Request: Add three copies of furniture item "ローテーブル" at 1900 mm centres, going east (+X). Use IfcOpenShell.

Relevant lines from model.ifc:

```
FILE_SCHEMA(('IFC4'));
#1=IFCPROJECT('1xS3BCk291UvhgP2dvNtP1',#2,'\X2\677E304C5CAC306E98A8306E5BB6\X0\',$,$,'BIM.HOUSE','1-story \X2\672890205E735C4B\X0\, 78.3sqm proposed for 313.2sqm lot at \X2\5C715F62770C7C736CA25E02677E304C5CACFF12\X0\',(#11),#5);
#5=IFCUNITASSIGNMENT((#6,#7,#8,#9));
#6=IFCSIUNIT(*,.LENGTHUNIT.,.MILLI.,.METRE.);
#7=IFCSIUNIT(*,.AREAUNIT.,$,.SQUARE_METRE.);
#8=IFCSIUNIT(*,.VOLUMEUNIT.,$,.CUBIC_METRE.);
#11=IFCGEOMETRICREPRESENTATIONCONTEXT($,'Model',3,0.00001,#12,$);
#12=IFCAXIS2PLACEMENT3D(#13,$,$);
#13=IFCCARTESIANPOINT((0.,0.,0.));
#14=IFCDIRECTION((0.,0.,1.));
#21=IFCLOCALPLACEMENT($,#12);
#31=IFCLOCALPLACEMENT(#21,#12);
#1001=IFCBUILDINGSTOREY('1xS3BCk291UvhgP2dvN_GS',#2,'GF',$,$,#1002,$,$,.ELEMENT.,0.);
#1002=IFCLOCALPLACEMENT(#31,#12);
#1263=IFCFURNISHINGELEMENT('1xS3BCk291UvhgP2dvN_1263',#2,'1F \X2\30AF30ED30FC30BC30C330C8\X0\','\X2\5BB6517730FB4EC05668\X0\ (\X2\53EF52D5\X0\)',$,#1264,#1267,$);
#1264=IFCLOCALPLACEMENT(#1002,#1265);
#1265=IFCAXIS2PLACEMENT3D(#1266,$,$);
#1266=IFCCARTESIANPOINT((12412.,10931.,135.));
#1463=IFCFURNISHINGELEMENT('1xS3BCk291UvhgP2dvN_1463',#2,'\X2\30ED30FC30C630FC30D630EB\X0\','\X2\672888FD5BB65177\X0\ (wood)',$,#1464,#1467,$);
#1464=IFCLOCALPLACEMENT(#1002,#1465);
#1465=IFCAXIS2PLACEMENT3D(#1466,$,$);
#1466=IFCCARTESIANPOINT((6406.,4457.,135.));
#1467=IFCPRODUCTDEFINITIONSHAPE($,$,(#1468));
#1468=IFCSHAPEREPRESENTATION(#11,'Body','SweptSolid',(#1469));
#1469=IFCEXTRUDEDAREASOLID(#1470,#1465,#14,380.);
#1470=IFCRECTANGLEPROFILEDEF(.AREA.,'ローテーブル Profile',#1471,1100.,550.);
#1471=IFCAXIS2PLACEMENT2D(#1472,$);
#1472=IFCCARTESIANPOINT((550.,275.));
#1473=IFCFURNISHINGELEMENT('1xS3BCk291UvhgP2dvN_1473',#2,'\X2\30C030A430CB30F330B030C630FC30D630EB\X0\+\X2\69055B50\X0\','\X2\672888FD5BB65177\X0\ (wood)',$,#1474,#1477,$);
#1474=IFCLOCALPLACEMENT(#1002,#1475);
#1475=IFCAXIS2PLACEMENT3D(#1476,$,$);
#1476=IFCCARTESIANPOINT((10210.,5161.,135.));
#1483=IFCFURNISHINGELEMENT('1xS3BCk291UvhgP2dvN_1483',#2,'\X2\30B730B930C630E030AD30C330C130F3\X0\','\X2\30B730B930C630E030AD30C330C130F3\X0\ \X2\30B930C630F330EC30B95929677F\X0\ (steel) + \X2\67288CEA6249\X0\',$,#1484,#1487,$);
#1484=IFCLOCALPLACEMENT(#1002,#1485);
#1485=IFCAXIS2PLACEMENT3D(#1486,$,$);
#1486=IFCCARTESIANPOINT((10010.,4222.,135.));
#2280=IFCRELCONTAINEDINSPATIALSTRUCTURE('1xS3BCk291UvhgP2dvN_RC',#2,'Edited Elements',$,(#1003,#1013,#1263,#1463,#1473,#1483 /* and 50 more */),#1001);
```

```python
import numpy as np
import ifcopenshell
import ifcopenshell.api.geometry
import ifcopenshell.api.root
import ifcopenshell.util.element
import ifcopenshell.util.placement

model = ifcopenshell.open("model.ifc")


def reuse_history(source, copy):
    """copy_class also copies each property set's owner history, people and application; keep the originals."""
    for rel in copy.IsDefinedBy:
        if rel.is_a("IfcRelDefinesByProperties") and (history := rel.RelatingPropertyDefinition.OwnerHistory):
            rel.RelatingPropertyDefinition.OwnerHistory = source.OwnerHistory
            ifcopenshell.util.element.remove_deep2(model, history)


source = model.by_guid("1xS3BCk291UvhgP2dvN_1463")
base = ifcopenshell.util.placement.get_local_placement(source.ObjectPlacement)
step = np.array([1.0, 0.0, 0.0]) * 1900.0

for i in range(1, 4):
    copy = ifcopenshell.api.root.copy_class(model, product=source)
    copy.Representation = ifcopenshell.util.element.copy_deep(
        model, source.Representation, exclude=["IfcGeometricRepresentationContext", "IfcRepresentationMap"]
    )
    reuse_history(source, copy)
    matrix = base.copy()
    matrix[:3, 3] += i * step
    print("added at", matrix[:3, 3].round(3) + 0.0)
    ifcopenshell.api.geometry.edit_object_placement(model, product=copy, matrix=matrix, is_si=False)

model.write("model_updated.ifc")
```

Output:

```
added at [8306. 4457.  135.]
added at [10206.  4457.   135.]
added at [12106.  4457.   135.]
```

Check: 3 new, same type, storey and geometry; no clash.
